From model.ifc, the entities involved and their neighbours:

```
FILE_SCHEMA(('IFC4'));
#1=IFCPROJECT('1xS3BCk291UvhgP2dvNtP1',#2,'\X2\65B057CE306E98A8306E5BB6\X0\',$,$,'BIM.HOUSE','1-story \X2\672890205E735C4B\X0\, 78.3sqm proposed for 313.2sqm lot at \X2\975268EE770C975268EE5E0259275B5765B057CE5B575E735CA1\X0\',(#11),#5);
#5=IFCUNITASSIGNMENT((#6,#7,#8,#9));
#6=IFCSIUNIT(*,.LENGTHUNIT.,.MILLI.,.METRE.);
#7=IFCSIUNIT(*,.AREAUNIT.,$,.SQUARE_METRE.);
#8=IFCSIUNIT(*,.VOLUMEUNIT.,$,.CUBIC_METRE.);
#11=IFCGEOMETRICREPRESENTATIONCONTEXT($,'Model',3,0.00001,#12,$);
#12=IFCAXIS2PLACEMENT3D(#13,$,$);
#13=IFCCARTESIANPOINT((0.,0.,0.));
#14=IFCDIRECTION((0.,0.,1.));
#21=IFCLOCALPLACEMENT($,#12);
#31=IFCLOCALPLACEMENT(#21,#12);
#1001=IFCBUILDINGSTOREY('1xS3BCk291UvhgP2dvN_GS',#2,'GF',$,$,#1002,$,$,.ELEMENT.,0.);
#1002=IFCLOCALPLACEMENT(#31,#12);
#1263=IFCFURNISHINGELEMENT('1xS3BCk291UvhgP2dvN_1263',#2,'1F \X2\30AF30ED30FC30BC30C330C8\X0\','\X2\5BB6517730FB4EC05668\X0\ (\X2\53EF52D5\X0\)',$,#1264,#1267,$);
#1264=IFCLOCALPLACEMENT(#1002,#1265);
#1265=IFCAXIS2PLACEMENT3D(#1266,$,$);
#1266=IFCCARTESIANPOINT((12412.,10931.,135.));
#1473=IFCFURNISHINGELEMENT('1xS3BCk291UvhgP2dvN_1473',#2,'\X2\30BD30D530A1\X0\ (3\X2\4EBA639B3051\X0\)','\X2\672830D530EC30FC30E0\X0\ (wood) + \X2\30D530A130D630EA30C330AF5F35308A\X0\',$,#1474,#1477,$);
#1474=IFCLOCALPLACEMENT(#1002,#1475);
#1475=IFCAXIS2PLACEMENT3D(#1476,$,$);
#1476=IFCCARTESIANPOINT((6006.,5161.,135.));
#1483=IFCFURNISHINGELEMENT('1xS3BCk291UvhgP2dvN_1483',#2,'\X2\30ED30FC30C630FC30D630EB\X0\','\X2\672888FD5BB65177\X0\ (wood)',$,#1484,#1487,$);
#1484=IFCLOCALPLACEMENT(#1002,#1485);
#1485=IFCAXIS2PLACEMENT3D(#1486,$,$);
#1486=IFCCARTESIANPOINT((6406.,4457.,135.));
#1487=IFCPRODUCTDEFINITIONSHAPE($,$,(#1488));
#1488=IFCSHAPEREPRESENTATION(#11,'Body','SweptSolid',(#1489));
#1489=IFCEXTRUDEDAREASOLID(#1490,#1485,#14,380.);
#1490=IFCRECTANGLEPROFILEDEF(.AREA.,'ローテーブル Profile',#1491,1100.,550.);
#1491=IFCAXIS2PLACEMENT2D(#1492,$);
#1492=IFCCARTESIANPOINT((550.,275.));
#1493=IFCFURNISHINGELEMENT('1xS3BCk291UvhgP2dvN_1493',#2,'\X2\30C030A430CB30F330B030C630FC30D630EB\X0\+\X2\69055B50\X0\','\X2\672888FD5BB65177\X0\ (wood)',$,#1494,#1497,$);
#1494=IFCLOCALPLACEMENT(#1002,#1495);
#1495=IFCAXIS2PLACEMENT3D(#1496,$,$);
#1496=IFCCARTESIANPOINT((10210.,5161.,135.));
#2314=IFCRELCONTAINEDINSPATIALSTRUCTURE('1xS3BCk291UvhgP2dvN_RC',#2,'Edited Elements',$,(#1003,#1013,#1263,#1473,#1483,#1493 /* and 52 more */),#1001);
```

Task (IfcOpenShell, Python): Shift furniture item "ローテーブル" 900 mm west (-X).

```python
import ifcopenshell
import ifcopenshell.api.geometry
import ifcopenshell.util.placement
import ifcopenshell.util.unit

model = ifcopenshell.open("model.ifc")
unit_scale = ifcopenshell.util.unit.calculate_unit_scale(model)

item = model.by_guid("1xS3BCk291UvhgP2dvN_1483")
matrix = ifcopenshell.util.placement.get_local_placement(item.ObjectPlacement)
matrix[0, 3] -= 0.9 / unit_scale
ifcopenshell.api.geometry.edit_object_placement(model, product=item, matrix=matrix, is_si=False)

print(ifcopenshell.util.placement.get_local_placement(item.ObjectPlacement).round(3) + 0.0)

model.write("model_v2.ifc")
```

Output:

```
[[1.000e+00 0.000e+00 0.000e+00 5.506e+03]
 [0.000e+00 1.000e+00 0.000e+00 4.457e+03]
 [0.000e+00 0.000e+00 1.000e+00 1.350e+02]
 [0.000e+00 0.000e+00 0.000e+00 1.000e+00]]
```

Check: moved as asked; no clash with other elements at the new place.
